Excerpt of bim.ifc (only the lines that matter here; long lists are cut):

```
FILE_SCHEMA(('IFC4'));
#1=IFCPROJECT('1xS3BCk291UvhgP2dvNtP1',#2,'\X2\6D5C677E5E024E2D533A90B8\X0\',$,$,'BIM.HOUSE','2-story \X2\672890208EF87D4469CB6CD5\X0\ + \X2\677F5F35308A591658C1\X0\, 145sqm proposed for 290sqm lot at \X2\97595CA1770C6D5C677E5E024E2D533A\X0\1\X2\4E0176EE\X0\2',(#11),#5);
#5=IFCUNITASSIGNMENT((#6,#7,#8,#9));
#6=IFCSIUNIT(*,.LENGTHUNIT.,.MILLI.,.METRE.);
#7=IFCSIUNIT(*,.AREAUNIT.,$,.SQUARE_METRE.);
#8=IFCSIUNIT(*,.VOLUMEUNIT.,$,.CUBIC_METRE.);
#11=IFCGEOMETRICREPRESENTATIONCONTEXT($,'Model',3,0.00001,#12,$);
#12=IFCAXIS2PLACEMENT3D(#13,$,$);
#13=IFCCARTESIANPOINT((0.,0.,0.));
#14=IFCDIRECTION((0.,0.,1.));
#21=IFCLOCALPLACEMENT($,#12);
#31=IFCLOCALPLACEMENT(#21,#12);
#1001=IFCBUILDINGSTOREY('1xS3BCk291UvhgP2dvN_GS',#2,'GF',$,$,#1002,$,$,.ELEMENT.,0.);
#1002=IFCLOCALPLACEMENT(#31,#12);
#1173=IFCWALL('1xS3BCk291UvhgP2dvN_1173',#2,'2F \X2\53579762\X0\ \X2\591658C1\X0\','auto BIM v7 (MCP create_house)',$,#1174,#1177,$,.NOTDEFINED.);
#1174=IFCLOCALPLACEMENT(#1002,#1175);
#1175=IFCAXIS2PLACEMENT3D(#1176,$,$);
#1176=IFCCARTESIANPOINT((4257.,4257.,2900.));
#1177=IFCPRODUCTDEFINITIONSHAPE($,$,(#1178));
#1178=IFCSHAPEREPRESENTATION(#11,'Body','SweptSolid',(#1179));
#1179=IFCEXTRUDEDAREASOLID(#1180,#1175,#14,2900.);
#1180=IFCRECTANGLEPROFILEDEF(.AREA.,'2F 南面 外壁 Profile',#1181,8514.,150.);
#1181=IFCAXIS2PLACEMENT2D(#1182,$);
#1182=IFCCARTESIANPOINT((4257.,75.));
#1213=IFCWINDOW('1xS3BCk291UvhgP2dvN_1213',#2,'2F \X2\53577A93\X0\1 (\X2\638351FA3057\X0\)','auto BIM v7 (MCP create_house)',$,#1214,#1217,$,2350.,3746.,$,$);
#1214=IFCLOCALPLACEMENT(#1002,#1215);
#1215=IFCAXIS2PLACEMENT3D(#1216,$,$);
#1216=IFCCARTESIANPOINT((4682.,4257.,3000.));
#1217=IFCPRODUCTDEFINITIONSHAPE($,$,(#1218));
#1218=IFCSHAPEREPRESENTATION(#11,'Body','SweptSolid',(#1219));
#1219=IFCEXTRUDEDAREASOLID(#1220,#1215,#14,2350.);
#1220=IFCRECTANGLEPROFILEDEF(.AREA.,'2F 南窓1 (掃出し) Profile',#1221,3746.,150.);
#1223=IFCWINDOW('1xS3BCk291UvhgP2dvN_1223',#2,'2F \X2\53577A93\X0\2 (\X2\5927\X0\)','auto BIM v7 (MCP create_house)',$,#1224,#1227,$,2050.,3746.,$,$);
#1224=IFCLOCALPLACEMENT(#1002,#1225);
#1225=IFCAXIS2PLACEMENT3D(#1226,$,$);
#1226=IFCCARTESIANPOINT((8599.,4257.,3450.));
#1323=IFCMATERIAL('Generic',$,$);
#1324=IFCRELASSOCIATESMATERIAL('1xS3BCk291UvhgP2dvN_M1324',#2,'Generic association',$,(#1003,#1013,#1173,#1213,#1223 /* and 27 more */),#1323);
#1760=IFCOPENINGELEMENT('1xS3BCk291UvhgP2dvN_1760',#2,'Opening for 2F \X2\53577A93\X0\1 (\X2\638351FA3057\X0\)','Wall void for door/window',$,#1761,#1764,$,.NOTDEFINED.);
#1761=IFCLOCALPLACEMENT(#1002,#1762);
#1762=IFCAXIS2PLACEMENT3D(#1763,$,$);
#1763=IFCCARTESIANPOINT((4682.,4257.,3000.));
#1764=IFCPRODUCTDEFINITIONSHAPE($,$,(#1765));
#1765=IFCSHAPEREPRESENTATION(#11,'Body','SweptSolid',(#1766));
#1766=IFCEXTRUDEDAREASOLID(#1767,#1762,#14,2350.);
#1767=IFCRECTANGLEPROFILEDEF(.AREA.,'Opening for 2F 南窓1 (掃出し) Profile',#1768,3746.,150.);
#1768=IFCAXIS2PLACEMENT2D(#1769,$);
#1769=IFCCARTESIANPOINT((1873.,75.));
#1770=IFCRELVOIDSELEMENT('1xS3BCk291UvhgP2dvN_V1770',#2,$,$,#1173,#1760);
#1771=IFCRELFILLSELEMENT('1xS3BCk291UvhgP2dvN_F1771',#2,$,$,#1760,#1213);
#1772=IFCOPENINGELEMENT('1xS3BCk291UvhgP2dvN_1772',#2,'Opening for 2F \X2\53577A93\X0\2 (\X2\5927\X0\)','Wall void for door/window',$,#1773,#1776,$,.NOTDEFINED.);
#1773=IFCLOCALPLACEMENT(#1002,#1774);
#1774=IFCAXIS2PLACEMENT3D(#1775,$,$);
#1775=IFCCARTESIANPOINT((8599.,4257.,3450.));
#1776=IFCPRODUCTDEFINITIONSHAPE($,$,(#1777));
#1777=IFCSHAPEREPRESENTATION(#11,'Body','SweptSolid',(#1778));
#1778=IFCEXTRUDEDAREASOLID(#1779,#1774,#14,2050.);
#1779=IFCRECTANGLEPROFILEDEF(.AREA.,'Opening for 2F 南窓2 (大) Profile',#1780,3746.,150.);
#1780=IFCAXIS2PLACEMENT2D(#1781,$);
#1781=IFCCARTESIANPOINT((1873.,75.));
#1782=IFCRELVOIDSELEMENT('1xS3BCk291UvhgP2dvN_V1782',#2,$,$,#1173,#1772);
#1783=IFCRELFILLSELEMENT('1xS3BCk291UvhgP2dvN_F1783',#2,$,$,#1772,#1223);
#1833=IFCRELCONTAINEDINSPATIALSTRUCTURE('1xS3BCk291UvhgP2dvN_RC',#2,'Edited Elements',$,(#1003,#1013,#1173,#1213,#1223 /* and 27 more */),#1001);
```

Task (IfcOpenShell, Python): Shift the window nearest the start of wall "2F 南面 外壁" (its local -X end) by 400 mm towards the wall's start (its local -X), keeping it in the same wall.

```python
import ifcopenshell
import ifcopenshell.api.geometry
import ifcopenshell.util.placement

model = ifcopenshell.open("bim.ifc")

window = model.by_guid("1xS3BCk291UvhgP2dvN_1213")
opening = window.FillsVoids[0].RelatingOpeningElement
wall = opening.VoidsElements[0].RelatingBuildingElement

wall_matrix = ifcopenshell.util.placement.get_local_placement(wall.ObjectPlacement)
shift = wall_matrix[:3, 0] * -400.0
before = ifcopenshell.util.placement.get_local_placement(window.ObjectPlacement)[:3, 3].copy()

# The window is not placed relative to its opening, so move both.
for product in (opening, window):
    matrix = ifcopenshell.util.placement.get_local_placement(product.ObjectPlacement)
    matrix[:3, 3] += shift
    ifcopenshell.api.geometry.edit_object_placement(model, product=product, matrix=matrix, is_si=False)

after = ifcopenshell.util.placement.get_local_placement(window.ObjectPlacement)[:3, 3]
print("window moved by", (after - before).round(3) + 0.0)

model.write("bim_updated.ifc")
```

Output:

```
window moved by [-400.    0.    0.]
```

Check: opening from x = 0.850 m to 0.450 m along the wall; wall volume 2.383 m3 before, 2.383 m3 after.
